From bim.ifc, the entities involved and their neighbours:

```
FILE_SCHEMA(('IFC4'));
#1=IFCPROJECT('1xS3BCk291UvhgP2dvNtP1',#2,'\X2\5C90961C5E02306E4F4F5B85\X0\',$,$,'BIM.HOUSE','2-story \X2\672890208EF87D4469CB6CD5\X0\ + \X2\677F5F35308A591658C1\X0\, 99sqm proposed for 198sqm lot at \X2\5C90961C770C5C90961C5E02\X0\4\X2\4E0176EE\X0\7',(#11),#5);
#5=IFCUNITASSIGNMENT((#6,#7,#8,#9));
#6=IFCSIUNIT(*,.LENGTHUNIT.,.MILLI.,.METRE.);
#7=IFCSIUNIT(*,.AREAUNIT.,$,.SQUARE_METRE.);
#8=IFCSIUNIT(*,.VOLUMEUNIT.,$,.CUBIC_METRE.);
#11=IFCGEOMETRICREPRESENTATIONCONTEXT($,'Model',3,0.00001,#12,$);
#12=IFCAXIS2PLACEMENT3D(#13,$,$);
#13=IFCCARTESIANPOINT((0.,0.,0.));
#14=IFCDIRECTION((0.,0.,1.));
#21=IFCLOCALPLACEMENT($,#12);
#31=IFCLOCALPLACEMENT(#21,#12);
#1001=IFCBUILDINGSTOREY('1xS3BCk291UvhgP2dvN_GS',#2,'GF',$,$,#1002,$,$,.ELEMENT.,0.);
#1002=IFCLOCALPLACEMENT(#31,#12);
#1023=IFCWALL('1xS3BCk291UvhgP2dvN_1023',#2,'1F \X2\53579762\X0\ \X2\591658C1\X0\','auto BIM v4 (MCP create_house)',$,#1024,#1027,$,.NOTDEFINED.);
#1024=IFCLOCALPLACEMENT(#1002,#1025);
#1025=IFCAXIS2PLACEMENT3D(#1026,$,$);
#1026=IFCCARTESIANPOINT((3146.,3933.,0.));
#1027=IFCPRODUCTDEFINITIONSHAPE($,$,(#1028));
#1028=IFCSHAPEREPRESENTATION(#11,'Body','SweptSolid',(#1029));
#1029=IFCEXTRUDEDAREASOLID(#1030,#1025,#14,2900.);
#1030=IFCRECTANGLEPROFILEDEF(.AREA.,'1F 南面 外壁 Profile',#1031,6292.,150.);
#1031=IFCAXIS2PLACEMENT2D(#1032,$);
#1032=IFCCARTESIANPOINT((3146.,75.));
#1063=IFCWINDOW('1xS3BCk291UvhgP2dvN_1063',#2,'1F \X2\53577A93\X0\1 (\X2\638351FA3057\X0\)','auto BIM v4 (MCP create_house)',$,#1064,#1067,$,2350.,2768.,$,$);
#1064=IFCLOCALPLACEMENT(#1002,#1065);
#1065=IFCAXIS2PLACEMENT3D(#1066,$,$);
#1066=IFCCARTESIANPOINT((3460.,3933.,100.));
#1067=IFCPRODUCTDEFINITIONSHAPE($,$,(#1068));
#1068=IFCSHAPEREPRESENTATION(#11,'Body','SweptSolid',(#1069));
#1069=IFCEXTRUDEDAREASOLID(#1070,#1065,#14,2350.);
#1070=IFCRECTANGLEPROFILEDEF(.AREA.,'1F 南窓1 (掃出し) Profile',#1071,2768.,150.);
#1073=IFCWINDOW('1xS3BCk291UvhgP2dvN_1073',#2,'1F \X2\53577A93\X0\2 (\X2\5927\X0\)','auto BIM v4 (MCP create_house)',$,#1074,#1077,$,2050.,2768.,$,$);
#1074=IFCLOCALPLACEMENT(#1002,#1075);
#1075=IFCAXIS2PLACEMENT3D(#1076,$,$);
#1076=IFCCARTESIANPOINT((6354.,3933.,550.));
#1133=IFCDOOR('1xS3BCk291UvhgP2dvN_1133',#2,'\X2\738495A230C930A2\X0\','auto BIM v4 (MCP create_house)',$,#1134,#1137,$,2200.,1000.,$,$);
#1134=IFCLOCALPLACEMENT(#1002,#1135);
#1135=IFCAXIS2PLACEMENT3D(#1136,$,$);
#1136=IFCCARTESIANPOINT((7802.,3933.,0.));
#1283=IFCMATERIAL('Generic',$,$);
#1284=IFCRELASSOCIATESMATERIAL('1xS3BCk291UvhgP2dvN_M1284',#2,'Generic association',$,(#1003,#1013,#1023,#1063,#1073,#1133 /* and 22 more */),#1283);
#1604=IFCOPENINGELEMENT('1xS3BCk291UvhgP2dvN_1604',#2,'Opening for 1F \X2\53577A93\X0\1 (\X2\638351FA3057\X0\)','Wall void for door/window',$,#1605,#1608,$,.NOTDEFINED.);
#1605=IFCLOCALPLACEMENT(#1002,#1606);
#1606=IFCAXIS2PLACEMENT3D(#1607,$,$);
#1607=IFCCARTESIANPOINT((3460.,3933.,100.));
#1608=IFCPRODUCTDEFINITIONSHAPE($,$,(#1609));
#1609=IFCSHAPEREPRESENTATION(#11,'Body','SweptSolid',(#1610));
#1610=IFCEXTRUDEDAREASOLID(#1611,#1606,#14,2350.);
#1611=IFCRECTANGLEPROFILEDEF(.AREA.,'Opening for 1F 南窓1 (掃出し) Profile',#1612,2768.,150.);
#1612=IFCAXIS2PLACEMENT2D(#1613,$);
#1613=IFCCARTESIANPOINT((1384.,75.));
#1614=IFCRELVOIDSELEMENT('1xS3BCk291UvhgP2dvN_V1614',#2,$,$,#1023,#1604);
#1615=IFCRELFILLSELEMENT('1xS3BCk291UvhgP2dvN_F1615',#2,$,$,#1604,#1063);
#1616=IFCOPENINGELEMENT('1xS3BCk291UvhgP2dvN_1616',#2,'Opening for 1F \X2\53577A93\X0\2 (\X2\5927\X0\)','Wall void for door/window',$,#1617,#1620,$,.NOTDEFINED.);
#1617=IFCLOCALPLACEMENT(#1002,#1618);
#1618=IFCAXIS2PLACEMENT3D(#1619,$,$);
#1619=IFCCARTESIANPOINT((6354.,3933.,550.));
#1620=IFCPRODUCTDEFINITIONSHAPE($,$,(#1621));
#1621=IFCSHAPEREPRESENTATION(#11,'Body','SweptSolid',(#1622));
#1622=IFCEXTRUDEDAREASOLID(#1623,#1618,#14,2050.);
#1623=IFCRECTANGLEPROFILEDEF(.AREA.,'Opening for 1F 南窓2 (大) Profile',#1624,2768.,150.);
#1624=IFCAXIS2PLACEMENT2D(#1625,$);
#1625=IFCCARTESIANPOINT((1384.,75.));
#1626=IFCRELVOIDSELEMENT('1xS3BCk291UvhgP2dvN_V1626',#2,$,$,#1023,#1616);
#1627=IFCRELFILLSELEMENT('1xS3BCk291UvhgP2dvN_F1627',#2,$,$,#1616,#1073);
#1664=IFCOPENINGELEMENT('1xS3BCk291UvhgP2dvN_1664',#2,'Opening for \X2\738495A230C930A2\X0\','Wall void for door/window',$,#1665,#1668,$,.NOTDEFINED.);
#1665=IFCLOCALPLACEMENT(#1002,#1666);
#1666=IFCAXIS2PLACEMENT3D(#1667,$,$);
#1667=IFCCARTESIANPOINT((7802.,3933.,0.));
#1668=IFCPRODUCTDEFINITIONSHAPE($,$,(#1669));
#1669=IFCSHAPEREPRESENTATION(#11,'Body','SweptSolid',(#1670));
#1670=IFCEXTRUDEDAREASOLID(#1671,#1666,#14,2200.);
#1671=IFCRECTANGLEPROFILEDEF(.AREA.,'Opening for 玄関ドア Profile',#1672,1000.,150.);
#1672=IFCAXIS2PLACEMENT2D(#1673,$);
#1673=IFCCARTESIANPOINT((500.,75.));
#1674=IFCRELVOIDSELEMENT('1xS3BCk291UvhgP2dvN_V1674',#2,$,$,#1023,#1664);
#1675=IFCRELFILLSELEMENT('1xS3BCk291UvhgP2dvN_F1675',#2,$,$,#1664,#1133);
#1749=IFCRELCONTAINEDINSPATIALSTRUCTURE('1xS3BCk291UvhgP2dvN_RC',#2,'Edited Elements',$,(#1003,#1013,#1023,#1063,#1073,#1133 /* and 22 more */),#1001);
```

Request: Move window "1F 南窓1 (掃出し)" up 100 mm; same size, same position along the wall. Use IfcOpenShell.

```python
import numpy as np
import ifcopenshell
import ifcopenshell.api.geometry
import ifcopenshell.util.placement
import ifcopenshell.util.unit

model = ifcopenshell.open("bim.ifc")
unit_scale = ifcopenshell.util.unit.calculate_unit_scale(model)

window = model.by_id(1063)
opening = window.FillsVoids[0].RelatingOpeningElement
dz = 100.0

shift = np.array([0.0, 0.0, dz])
# The window is not placed relative to its opening, so move both.
for product in (opening, window):
    matrix = ifcopenshell.util.placement.get_local_placement(product.ObjectPlacement)
    matrix[:3, 3] += shift
    ifcopenshell.api.geometry.edit_object_placement(model, product=product, matrix=matrix, is_si=False)

print(f"moved by {dz * unit_scale:+.3f} m")

model.write("bim-out.ifc")
```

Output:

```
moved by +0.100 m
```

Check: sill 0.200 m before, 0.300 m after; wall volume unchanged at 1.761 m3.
